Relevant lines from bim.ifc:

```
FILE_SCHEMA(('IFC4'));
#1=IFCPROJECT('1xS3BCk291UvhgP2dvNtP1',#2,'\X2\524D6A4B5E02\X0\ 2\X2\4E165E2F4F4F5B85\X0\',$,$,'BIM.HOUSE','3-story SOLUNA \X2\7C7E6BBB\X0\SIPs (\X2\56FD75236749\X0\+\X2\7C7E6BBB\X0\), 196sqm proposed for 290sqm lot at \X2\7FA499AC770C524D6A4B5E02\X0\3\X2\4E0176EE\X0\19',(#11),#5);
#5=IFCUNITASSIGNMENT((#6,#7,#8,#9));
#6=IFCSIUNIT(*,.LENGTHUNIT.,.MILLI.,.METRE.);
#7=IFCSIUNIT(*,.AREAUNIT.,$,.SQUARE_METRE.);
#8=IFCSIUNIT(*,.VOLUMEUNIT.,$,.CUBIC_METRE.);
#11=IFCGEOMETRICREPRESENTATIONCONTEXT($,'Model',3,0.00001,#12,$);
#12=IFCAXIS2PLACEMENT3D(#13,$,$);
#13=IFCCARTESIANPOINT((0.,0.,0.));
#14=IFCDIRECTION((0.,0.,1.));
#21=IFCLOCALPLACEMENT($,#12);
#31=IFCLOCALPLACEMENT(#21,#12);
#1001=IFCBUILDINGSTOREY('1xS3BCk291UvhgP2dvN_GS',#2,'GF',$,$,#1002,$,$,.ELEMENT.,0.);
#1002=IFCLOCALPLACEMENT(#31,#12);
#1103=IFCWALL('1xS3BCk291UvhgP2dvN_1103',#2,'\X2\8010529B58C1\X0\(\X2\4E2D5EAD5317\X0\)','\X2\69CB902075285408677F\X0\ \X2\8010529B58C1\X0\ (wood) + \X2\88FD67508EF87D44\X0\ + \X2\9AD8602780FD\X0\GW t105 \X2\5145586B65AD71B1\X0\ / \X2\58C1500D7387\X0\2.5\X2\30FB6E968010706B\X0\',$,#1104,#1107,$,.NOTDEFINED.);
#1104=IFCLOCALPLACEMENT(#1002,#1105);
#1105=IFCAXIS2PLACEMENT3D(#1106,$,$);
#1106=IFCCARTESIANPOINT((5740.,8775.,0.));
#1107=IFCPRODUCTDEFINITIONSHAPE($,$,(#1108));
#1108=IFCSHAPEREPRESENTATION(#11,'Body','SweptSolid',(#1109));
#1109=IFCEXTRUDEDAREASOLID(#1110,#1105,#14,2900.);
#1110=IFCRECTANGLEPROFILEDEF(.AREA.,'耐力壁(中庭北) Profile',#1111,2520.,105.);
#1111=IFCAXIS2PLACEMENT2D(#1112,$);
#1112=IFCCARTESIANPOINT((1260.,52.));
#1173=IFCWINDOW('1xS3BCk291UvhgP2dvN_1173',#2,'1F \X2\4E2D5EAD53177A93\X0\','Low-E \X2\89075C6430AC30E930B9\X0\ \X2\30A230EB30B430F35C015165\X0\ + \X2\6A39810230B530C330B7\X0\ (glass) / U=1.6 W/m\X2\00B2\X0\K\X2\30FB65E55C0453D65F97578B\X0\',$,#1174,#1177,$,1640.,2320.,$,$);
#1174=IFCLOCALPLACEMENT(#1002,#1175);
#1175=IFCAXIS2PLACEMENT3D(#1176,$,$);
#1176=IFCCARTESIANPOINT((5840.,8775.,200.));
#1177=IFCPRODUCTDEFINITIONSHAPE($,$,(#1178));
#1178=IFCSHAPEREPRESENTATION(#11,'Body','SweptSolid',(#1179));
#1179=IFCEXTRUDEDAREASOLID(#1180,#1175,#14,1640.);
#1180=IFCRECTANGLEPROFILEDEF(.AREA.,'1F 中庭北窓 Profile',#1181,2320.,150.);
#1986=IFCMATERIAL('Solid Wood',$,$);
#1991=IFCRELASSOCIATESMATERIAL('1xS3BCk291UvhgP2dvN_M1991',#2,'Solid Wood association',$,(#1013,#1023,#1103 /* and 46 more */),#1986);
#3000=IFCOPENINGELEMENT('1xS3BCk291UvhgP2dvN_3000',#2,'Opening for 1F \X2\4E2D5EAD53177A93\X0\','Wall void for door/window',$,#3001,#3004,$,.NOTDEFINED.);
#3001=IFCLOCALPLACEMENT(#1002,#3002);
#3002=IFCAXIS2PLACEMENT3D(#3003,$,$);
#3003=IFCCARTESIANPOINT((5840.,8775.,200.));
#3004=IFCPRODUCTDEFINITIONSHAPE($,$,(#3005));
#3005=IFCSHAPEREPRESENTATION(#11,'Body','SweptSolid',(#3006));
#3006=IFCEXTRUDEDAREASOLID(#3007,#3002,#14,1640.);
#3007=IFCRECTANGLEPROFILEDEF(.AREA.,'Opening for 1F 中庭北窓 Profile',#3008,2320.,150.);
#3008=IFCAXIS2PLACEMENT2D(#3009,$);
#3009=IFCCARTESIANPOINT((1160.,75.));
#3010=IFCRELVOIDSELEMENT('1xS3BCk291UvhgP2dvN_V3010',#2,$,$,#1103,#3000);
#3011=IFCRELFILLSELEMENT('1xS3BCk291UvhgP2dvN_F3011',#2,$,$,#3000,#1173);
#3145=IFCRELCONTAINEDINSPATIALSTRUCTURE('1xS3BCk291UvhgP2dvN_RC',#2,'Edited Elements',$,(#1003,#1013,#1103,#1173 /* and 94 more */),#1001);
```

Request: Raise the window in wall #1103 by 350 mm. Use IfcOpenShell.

```python
import numpy as np
import ifcopenshell
import ifcopenshell.api.geometry
import ifcopenshell.util.placement
import ifcopenshell.util.unit

model = ifcopenshell.open("bim.ifc")
unit_scale = ifcopenshell.util.unit.calculate_unit_scale(model)

window = model.by_guid("1xS3BCk291UvhgP2dvN_1173")
opening = window.FillsVoids[0].RelatingOpeningElement
dz = 0.35 / unit_scale

shift = np.array([0.0, 0.0, dz])
# The window is not placed relative to its opening, so move both.
for product in (opening, window):
    matrix = ifcopenshell.util.placement.get_local_placement(product.ObjectPlacement)
    matrix[:3, 3] += shift
    ifcopenshell.api.geometry.edit_object_placement(model, product=product, matrix=matrix, is_si=False)

print(f"moved by {dz * unit_scale:+.3f} m")

model.write("bim-out.ifc")
```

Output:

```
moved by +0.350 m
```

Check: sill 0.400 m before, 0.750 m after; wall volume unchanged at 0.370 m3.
